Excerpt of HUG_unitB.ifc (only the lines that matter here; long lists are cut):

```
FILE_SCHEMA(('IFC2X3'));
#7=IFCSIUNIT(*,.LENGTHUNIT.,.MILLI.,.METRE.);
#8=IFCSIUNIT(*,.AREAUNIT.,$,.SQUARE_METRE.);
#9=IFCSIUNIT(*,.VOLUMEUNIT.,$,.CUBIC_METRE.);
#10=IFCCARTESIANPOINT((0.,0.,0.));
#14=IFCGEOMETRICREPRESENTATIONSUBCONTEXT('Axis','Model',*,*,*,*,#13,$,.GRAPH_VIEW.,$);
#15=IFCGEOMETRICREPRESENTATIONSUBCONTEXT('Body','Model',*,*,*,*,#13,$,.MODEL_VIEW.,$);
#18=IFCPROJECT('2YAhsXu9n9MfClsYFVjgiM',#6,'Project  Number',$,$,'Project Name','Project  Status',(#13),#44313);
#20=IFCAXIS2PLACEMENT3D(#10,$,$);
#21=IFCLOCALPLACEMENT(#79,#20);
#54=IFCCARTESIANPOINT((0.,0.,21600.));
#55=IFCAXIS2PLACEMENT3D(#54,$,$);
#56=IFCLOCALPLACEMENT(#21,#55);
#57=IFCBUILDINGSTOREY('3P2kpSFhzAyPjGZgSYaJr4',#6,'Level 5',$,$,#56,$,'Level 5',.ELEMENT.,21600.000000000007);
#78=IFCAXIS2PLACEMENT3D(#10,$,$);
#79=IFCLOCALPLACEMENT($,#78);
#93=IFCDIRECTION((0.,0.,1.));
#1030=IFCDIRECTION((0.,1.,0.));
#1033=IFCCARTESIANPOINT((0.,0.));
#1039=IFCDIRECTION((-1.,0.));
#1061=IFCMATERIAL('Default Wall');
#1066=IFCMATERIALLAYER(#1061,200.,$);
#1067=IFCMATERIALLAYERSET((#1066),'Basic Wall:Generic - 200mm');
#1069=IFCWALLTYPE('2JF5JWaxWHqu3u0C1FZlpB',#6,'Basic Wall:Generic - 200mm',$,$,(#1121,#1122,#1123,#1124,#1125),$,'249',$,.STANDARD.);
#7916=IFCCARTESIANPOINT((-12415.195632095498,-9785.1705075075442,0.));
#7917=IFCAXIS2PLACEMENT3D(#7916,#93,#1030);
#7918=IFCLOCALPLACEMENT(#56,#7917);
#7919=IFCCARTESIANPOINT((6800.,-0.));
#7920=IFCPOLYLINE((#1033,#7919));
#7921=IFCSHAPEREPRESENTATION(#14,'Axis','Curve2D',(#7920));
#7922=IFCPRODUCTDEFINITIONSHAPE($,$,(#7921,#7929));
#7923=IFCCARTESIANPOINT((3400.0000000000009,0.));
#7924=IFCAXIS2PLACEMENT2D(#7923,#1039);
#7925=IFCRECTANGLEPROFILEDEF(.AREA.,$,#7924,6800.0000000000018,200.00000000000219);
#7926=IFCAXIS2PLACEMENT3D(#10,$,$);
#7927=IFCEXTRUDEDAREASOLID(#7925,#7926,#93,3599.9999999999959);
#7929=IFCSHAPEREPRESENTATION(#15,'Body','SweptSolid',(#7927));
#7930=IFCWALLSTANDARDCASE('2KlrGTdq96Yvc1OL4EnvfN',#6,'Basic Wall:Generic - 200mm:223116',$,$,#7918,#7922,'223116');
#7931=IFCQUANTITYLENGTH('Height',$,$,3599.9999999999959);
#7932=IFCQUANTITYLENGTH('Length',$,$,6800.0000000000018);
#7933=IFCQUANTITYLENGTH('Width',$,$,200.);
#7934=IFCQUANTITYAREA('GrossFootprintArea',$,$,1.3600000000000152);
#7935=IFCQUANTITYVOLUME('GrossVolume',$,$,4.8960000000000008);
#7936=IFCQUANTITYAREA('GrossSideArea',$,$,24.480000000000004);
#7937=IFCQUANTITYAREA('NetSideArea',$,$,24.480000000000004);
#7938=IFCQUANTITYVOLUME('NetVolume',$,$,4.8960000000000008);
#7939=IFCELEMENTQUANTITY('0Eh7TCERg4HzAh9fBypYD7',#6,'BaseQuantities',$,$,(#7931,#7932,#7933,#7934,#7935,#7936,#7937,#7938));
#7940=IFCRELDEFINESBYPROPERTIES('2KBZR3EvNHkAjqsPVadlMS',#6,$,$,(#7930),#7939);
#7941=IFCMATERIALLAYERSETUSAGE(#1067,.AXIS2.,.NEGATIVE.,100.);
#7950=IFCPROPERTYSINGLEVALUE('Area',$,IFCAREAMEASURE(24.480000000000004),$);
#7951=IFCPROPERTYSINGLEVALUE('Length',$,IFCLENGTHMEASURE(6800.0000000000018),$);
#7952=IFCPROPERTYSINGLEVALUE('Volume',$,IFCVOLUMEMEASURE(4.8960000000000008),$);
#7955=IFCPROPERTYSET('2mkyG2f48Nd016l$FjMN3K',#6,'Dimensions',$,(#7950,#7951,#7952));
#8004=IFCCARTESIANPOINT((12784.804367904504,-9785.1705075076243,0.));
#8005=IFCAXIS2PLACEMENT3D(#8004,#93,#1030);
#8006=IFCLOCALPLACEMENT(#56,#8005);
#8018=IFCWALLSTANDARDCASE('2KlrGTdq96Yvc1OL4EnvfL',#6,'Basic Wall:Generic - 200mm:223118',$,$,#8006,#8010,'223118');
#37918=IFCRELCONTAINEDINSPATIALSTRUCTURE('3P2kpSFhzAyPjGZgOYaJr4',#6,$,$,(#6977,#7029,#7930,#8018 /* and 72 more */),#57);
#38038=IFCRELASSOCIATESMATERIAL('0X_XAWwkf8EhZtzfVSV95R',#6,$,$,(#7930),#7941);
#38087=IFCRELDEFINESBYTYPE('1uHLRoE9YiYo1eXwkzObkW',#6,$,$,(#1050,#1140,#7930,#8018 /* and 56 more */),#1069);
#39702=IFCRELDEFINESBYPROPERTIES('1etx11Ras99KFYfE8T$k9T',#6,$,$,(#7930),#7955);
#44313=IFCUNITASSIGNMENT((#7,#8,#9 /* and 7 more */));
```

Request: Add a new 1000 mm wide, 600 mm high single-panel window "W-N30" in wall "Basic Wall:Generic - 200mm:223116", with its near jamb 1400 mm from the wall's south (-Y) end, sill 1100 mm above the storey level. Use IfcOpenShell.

```python
import numpy as np
import ifcopenshell
import ifcopenshell.api.feature
import ifcopenshell.api.geometry
import ifcopenshell.api.pset
import ifcopenshell.api.root
import ifcopenshell.api.spatial
import ifcopenshell.api.type
import ifcopenshell.geom
import ifcopenshell.util.element
import ifcopenshell.util.placement
import ifcopenshell.util.representation
import ifcopenshell.util.shape
import ifcopenshell.util.unit

model = ifcopenshell.open("HUG_unitB.ifc")
unit_scale = ifcopenshell.util.unit.calculate_unit_scale(model)
area_scale = ifcopenshell.util.unit.calculate_unit_scale(model, "AREAUNIT")
volume_scale = ifcopenshell.util.unit.calculate_unit_scale(model, "VOLUMEUNIT")
settings = ifcopenshell.geom.settings()


def volume(element):
    """Net volume in cubic metres, openings subtracted."""
    shape = ifcopenshell.geom.create_shape(settings, element)
    return ifcopenshell.util.shape.get_volume(shape.geometry)


wall = model.by_guid("2KlrGTdq96Yvc1OL4EnvfN")
storey = ifcopenshell.util.element.get_container(wall, ifc_class="IfcBuildingStorey")
context = ifcopenshell.util.representation.get_context(model, "Model", "Body", "MODEL_VIEW")
before = volume(wall)

width, height, from_end, sill = 1, 0.6, 1.4, 1.1  # metres

# The wall runs along its own X axis, and the end named is its -X end.
wall_shape = ifcopenshell.geom.create_shape(settings, wall)
x, y, z = ifcopenshell.util.shape.get_vertices(wall_shape.geometry).T
start = x.min() + from_end
face, thickness = float(y.min()), float(y.max() - y.min())
wall_matrix = ifcopenshell.util.placement.get_local_placement(wall.ObjectPlacement)
level = ifcopenshell.util.placement.get_local_placement(storey.ObjectPlacement)[2, 3]


def in_wall(x, y):
    """Placement at x, y metres in the wall's axes, at sill height."""
    matrix = wall_matrix.copy()
    matrix[:, 3] = wall_matrix @ np.array([x / unit_scale, y / unit_scale, 0.0, 1.0])
    matrix[2, 3] = level + sill / unit_scale
    return matrix


# Opening: a box that overshoots both wall faces by 50 mm.
opening = ifcopenshell.api.root.create_entity(model, ifc_class="IfcOpeningElement")
box = ifcopenshell.api.geometry.add_wall_representation(
    model, context=context, length=width, height=height, thickness=thickness + 0.1
)
ifcopenshell.api.geometry.assign_representation(model, product=opening, representation=box)
ifcopenshell.api.geometry.edit_object_placement(model, product=opening, matrix=in_wall(start, face - 0.05), is_si=False)
ifcopenshell.api.feature.add_feature(model, feature=opening, element=wall)

window = ifcopenshell.api.root.create_entity(model, ifc_class="IfcWindow", name="W-N30")
window.OverallWidth, window.OverallHeight = width / unit_scale, height / unit_scale
body = ifcopenshell.api.geometry.add_window_representation(
    model,
    context=context,
    overall_width=window.OverallWidth,
    overall_height=window.OverallHeight,
    partition_type="SINGLE_PANEL",
)
ifcopenshell.api.geometry.assign_representation(model, product=window, representation=body)
ifcopenshell.api.spatial.assign_container(model, products=[window], relating_structure=storey)
fills = ifcopenshell.api.feature.add_filling(model, opening=opening, element=window)
fills.OwnerHistory = window.OwnerHistory  # required in IFC2X3

# IFC2X3 keeps the operation on the window style.
style = ifcopenshell.api.root.create_entity(model, ifc_class="IfcWindowStyle", name="W-N30")
style.OperationType, style.ConstructionType = "SINGLE_PANEL", "NOTDEFINED"
style.ParameterTakesPrecedence = style.Sizeable = False
ifcopenshell.api.type.assign_type(model, related_objects=[window], relating_type=style)

# Centre the window in the wall's thickness.
ifcopenshell.api.geometry.edit_object_placement(model, product=window, matrix=in_wall(start, face), is_si=False)
window_shape = ifcopenshell.geom.create_shape(settings, window)
depth = ifcopenshell.util.shape.get_vertices(window_shape.geometry)[:, 1]
offset = face + thickness / 2 - (depth.min() + depth.max()) / 2
ifcopenshell.api.geometry.edit_object_placement(model, product=window, matrix=in_wall(start, offset), is_si=False)

after = volume(wall)

# Update the wall's stored quantities.
qto = model.by_id(ifcopenshell.util.element.get_pset(wall, "BaseQuantities", should_inherit=False)["id"])
ifcopenshell.api.pset.edit_qto(model, qto=qto, properties={
    "NetSideArea": after / thickness / area_scale,
    "NetVolume": after / volume_scale,
})
pset = model.by_id(ifcopenshell.util.element.get_pset(wall, "Dimensions", should_inherit=False)["id"])
ifcopenshell.api.pset.edit_pset(model, pset=pset, properties={
    "Area": model.create_entity("IfcAreaMeasure", after / thickness / area_scale),
    "Volume": model.create_entity("IfcVolumeMeasure", after / volume_scale),
})

print(f"wall volume {before:.3f} -> {after:.3f} m3")

model.write("HUG_unitB_v2.ifc")
```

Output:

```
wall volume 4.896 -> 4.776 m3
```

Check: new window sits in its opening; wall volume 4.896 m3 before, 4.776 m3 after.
